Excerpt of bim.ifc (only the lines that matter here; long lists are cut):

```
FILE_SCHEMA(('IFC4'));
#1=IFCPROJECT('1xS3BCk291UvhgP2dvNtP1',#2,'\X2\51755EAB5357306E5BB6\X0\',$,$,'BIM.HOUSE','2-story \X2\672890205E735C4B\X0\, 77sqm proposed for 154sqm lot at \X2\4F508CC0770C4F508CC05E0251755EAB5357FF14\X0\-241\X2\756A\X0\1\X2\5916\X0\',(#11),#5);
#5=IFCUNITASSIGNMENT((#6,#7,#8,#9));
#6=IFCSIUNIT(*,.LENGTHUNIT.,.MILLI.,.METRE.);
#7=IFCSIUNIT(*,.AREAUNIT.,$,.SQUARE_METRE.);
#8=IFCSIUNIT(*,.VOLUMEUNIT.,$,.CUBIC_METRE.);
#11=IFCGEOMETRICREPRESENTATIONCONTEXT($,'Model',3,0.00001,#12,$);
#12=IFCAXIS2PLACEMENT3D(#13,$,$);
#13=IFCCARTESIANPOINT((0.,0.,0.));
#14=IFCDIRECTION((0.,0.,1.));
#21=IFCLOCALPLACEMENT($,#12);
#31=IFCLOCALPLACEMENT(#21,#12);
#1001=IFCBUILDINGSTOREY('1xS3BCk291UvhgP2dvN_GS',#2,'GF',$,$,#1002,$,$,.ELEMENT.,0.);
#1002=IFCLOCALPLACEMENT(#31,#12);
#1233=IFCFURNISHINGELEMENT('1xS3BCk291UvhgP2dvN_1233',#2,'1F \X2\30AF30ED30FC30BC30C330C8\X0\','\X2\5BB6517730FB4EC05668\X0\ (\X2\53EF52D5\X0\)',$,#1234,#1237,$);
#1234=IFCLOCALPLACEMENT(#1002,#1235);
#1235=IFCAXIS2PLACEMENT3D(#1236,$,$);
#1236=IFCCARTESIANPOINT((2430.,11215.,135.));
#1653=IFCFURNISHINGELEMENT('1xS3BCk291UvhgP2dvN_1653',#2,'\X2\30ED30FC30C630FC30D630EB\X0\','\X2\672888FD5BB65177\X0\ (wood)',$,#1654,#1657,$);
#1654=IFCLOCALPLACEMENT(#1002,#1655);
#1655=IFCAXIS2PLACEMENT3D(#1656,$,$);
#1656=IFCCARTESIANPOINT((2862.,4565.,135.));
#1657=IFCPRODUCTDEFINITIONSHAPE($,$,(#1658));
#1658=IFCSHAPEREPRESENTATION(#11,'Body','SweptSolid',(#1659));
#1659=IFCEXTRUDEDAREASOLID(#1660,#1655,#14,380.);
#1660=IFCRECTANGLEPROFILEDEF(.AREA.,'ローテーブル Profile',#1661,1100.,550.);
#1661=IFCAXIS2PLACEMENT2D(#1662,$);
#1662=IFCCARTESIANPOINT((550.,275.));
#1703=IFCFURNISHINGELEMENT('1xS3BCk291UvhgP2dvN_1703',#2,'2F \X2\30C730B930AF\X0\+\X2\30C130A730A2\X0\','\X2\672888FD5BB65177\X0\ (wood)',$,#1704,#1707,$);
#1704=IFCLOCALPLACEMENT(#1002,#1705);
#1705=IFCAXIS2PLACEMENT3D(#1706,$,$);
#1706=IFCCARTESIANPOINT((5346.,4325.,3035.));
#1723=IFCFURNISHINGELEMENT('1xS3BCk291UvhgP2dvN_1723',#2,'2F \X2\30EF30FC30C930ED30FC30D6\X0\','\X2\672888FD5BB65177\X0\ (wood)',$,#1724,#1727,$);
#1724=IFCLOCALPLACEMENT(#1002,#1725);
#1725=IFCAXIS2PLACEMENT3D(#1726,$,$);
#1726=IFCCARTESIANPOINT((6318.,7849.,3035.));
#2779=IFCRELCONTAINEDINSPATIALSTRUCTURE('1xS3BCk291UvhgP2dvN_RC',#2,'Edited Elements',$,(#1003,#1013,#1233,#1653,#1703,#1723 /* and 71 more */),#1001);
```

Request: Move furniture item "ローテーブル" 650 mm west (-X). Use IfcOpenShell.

```python
import ifcopenshell
import ifcopenshell.api.geometry
import ifcopenshell.util.placement
import ifcopenshell.util.unit

model = ifcopenshell.open("bim.ifc")
unit_scale = ifcopenshell.util.unit.calculate_unit_scale(model)

item = model.by_guid("1xS3BCk291UvhgP2dvN_1653")
matrix = ifcopenshell.util.placement.get_local_placement(item.ObjectPlacement)
matrix[0, 3] -= 0.65 / unit_scale
ifcopenshell.api.geometry.edit_object_placement(model, product=item, matrix=matrix, is_si=False)

print(ifcopenshell.util.placement.get_local_placement(item.ObjectPlacement).round(3) + 0.0)

model.write("bim_edited.ifc")
```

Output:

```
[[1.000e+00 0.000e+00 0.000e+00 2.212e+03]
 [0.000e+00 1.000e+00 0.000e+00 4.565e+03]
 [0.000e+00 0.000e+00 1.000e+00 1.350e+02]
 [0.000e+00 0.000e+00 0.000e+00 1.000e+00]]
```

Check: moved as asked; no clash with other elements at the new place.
